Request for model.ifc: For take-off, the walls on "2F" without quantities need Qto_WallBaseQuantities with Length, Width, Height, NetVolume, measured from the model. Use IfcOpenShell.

First a look at what the model holds.

```python
import ifcopenshell
import ifcopenshell.util.element
import ifcopenshell.util.unit

model = ifcopenshell.open("model.ifc")
print(model.schema)
for unit_type in ("LENGTHUNIT", "AREAUNIT", "VOLUMEUNIT"):
    print(unit_type, ifcopenshell.util.unit.calculate_unit_scale(model, unit_type))
storey = next(s for s in model.by_type("IfcBuildingStorey") if s.Name == "2F")
walls = [e for e in ifcopenshell.util.element.get_decomposition(storey) if e.is_a("IfcWall")]
for e in sorted(walls, key=lambda e: e.id()):
    print(e.id(), e.is_a(), e.Name, list(ifcopenshell.util.element.get_psets(e, qtos_only=True)), sep=" | ")
```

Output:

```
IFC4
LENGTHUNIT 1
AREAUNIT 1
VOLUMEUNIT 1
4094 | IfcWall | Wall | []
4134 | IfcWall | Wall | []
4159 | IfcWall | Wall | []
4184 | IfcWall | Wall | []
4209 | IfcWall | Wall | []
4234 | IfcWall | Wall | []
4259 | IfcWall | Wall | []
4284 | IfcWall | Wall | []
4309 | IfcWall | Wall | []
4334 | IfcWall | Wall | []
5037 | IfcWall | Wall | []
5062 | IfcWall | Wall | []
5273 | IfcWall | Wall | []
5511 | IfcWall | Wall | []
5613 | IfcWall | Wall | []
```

```python
import ifcopenshell
import ifcopenshell.api.pset
import ifcopenshell.geom
import ifcopenshell.util.element
import ifcopenshell.util.shape
import ifcopenshell.util.unit

model = ifcopenshell.open("model.ifc")
unit_scale = ifcopenshell.util.unit.calculate_unit_scale(model)
volume_scale = ifcopenshell.util.unit.calculate_unit_scale(model, "VOLUMEUNIT")
settings = ifcopenshell.geom.settings()

storey = next(s for s in model.by_type("IfcBuildingStorey") if s.Name == "2F")
walls = [e for e in ifcopenshell.util.element.get_decomposition(storey) if e.is_a("IfcWall")]

for e in sorted(walls, key=lambda e: e.id()):
    if ifcopenshell.util.element.get_psets(e, qtos_only=True, should_inherit=False):
        continue
    # Geometry comes back in metres, in the element's own axes.
    shape = ifcopenshell.geom.create_shape(settings, e)
    values = {
        "Length": ifcopenshell.util.shape.get_x(shape.geometry) / unit_scale,
        "Width": ifcopenshell.util.shape.get_y(shape.geometry) / unit_scale,
        "Height": ifcopenshell.util.shape.get_z(shape.geometry) / unit_scale,
        "NetVolume": ifcopenshell.util.shape.get_volume(shape.geometry) / volume_scale,
    }
    qto = ifcopenshell.api.pset.add_qto(model, product=e, name="Qto_WallBaseQuantities")
    ifcopenshell.api.pset.edit_qto(model, qto=qto, properties=values)
    print(e.id(), {k: round(v, 3) for k, v in values.items()})

model.write("model_edited.ifc")
```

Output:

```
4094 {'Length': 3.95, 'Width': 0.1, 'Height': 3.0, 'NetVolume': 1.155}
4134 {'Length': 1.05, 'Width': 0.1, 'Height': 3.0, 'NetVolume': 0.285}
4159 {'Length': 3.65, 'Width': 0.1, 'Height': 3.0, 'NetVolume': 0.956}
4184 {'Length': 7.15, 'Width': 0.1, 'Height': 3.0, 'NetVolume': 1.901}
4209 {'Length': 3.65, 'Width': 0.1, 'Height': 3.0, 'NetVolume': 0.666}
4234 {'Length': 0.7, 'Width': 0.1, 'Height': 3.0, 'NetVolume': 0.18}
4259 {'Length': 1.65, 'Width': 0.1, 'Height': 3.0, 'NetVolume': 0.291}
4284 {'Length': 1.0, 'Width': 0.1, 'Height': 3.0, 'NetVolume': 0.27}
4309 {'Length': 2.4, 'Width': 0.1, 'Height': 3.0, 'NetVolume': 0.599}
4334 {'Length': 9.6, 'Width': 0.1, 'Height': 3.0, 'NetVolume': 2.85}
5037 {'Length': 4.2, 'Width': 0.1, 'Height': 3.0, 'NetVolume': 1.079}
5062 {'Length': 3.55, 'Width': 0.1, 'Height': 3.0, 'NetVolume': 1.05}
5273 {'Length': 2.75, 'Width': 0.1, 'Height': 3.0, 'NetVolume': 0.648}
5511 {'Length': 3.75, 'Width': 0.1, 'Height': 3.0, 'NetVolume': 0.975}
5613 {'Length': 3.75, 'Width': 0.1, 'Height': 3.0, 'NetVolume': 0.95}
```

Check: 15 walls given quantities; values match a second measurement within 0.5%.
